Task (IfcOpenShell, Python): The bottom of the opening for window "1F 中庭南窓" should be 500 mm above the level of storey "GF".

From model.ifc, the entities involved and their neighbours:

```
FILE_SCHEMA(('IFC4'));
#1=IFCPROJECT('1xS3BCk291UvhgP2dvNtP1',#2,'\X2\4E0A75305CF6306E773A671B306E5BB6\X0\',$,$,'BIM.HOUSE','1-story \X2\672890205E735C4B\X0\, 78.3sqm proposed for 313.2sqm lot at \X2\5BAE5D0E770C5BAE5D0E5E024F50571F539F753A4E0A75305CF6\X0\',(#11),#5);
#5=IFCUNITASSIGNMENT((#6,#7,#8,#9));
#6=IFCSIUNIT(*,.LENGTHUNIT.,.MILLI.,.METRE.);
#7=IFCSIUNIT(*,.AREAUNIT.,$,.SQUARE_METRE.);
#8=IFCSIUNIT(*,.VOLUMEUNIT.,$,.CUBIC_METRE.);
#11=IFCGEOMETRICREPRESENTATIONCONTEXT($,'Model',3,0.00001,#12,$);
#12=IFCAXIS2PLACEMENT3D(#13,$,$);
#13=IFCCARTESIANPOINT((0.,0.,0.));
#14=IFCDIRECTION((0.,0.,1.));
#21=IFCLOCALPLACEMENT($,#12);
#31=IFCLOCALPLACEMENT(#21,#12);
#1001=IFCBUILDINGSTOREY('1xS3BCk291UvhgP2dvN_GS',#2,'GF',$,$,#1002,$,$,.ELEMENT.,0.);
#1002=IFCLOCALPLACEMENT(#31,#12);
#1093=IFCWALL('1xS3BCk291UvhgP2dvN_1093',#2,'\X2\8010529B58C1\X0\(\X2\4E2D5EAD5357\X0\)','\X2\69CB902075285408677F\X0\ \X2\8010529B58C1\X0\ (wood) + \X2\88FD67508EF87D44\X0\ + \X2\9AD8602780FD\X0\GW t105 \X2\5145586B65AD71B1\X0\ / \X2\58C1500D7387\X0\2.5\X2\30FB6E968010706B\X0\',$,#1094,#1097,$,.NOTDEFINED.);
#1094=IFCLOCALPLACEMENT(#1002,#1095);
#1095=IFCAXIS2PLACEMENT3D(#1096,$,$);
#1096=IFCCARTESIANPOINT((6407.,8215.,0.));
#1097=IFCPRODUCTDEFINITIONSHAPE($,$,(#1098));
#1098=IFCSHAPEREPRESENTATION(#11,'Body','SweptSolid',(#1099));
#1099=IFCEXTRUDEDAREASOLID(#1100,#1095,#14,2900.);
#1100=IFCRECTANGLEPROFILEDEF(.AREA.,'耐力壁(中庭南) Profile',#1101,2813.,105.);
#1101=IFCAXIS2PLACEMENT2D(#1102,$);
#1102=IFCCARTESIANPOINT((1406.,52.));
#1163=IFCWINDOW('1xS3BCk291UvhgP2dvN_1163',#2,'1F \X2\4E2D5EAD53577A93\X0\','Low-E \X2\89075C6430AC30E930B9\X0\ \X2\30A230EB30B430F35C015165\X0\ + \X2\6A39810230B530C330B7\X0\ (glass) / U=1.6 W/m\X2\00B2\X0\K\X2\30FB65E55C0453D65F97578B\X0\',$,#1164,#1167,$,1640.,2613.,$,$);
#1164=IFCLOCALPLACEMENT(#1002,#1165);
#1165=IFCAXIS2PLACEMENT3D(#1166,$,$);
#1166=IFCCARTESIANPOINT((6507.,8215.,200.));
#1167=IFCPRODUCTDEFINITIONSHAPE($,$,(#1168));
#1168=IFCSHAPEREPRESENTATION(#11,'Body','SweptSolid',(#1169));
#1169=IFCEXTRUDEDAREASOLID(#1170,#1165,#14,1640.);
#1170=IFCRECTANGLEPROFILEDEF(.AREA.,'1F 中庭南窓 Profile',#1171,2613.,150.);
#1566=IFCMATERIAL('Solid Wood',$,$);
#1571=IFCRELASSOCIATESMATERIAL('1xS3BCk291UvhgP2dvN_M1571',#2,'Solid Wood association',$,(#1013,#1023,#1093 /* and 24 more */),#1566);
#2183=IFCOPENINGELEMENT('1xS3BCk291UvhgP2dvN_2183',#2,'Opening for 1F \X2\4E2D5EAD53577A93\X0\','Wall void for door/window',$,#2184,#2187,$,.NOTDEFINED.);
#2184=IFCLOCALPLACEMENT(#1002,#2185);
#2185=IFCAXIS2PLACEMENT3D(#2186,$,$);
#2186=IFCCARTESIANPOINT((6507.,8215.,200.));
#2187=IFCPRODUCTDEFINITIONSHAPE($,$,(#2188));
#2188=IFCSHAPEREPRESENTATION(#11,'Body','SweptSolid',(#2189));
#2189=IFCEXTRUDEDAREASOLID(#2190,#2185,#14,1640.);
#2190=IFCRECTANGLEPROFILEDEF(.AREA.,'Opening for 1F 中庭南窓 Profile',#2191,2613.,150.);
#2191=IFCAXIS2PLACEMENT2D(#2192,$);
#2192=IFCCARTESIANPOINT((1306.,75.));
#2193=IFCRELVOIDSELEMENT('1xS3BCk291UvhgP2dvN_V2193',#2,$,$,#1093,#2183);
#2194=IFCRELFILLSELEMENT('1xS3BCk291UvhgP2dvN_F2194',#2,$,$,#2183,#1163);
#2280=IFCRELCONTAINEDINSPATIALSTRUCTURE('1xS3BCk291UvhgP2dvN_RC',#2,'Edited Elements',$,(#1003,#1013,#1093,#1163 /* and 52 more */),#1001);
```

```python
import numpy as np
import ifcopenshell
import ifcopenshell.api.geometry
import ifcopenshell.geom
import ifcopenshell.util.element
import ifcopenshell.util.placement
import ifcopenshell.util.shape
import ifcopenshell.util.unit

model = ifcopenshell.open("model.ifc")
unit_scale = ifcopenshell.util.unit.calculate_unit_scale(model)

window = model.by_guid("1xS3BCk291UvhgP2dvN_1163")
opening = window.FillsVoids[0].RelatingOpeningElement
storey = ifcopenshell.util.element.get_container(window, ifc_class="IfcBuildingStorey")
level = ifcopenshell.util.placement.get_local_placement(storey.ObjectPlacement)[2, 3]

# The opening's origin need not be at the sill, so measure its lowest point.
shape = ifcopenshell.geom.create_shape(ifcopenshell.geom.settings(), opening)
bottom = ifcopenshell.util.shape.get_shape_bottom_elevation(shape, shape.geometry) / unit_scale
dz = level + 0.5 / unit_scale - bottom

shift = np.array([0.0, 0.0, dz])
# The window is not placed relative to its opening, so move both.
for product in (opening, window):
    matrix = ifcopenshell.util.placement.get_local_placement(product.ObjectPlacement)
    matrix[:3, 3] += shift
    ifcopenshell.api.geometry.edit_object_placement(model, product=product, matrix=matrix, is_si=False)

print(f"moved by {dz * unit_scale:+.3f} m")

model.write("model-out.ifc")
```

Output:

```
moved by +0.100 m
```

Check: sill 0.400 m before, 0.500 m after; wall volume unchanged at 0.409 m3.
